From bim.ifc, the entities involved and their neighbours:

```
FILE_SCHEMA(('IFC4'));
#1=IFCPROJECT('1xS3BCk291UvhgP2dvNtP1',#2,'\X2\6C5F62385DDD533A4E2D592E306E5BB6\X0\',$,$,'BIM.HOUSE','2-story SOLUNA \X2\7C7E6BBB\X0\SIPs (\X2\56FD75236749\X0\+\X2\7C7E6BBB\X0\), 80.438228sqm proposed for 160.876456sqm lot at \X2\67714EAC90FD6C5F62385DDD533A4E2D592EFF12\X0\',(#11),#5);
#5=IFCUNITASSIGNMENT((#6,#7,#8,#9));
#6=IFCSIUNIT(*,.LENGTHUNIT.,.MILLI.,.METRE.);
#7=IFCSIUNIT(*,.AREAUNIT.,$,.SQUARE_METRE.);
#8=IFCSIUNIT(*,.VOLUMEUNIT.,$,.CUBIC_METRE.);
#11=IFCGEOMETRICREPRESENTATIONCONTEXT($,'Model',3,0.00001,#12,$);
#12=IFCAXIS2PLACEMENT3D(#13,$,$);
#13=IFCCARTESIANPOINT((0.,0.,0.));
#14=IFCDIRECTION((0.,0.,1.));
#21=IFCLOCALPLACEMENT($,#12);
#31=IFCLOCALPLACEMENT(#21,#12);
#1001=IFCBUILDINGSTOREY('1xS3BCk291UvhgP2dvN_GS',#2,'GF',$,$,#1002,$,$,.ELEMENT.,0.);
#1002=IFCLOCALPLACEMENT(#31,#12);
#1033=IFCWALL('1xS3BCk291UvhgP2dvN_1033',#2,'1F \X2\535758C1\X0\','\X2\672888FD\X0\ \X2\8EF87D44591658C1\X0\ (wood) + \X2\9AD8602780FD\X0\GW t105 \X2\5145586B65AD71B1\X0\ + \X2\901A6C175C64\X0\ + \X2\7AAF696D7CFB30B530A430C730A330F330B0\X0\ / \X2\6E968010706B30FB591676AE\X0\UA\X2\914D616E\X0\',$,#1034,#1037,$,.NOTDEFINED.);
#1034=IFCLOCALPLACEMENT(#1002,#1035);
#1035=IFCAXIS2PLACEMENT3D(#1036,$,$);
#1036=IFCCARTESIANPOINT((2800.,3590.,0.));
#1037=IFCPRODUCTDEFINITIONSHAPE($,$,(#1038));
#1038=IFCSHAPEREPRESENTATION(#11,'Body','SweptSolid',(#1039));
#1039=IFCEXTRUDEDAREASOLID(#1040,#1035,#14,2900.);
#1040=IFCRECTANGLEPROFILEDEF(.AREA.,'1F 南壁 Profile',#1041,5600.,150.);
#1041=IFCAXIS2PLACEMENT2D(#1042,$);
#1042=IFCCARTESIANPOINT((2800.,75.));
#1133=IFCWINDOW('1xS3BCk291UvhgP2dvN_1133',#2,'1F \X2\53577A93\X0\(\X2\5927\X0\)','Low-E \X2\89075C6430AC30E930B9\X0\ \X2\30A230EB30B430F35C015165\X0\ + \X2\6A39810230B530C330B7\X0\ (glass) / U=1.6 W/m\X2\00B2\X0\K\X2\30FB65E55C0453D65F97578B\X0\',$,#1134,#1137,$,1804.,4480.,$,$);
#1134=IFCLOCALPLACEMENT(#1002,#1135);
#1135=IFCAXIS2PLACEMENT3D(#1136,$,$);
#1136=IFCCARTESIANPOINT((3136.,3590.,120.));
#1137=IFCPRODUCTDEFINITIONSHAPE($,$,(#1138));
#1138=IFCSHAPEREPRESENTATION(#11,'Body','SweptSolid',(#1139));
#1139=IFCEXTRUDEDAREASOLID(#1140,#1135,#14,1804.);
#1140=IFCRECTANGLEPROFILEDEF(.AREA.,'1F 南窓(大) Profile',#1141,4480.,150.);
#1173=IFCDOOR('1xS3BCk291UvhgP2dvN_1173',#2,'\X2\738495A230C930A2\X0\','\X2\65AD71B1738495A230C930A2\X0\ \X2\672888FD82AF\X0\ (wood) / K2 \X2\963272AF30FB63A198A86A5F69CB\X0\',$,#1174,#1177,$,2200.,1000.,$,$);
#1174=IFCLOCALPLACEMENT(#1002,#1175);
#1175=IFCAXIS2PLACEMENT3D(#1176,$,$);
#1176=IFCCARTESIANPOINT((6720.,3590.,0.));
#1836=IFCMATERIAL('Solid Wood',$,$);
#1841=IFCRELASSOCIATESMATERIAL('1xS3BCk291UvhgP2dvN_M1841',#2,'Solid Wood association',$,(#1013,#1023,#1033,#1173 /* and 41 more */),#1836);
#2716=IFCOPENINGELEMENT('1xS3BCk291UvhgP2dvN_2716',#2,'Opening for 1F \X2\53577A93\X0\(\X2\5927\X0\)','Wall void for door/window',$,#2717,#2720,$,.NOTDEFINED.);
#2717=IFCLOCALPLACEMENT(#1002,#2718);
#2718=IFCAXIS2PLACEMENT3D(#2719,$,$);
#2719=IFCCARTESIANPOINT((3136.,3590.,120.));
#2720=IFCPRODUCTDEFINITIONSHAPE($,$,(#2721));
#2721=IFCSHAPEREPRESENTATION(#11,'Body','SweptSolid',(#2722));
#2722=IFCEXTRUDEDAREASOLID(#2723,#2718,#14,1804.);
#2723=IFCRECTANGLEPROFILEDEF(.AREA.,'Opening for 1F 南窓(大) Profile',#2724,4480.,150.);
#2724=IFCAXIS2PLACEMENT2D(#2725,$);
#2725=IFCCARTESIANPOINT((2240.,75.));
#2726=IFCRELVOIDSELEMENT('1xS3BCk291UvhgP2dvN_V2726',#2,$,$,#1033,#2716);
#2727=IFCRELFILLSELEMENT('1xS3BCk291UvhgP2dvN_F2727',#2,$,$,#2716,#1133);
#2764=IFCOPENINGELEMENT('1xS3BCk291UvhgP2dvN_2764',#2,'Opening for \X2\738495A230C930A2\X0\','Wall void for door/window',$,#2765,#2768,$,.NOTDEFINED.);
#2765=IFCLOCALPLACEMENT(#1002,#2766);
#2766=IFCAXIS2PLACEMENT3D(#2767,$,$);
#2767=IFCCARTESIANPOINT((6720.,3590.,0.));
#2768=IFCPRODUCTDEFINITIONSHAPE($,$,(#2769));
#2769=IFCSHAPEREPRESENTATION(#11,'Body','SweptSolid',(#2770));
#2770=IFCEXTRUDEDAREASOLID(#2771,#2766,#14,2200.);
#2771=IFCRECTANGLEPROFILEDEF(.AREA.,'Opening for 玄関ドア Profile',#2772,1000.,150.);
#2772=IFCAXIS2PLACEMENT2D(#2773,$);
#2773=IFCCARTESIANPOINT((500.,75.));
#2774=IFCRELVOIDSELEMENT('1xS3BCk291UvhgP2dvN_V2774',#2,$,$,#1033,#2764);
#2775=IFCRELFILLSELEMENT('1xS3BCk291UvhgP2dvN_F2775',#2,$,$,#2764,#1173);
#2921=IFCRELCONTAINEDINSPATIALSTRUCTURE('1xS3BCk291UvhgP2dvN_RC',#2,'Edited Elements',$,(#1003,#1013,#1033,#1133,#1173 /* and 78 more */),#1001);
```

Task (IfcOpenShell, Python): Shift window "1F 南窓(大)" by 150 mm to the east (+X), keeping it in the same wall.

```python
import ifcopenshell
import ifcopenshell.api.geometry
import ifcopenshell.util.placement

model = ifcopenshell.open("bim.ifc")

window = model.by_id(1133)
opening = window.FillsVoids[0].RelatingOpeningElement
wall = opening.VoidsElements[0].RelatingBuildingElement

wall_matrix = ifcopenshell.util.placement.get_local_placement(wall.ObjectPlacement)
shift = wall_matrix[:3, 0] * 150.0
before = ifcopenshell.util.placement.get_local_placement(window.ObjectPlacement)[:3, 3].copy()

# The window is not placed relative to its opening, so move both.
for product in (opening, window):
    matrix = ifcopenshell.util.placement.get_local_placement(product.ObjectPlacement)
    matrix[:3, 3] += shift
    ifcopenshell.api.geometry.edit_object_placement(model, product=product, matrix=matrix, is_si=False)

after = ifcopenshell.util.placement.get_local_placement(window.ObjectPlacement)[:3, 3]
print("window moved by", (after - before).round(3) + 0.0)

model.write("bim-out.ifc")
```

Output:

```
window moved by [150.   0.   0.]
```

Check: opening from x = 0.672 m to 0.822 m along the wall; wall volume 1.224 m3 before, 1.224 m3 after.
